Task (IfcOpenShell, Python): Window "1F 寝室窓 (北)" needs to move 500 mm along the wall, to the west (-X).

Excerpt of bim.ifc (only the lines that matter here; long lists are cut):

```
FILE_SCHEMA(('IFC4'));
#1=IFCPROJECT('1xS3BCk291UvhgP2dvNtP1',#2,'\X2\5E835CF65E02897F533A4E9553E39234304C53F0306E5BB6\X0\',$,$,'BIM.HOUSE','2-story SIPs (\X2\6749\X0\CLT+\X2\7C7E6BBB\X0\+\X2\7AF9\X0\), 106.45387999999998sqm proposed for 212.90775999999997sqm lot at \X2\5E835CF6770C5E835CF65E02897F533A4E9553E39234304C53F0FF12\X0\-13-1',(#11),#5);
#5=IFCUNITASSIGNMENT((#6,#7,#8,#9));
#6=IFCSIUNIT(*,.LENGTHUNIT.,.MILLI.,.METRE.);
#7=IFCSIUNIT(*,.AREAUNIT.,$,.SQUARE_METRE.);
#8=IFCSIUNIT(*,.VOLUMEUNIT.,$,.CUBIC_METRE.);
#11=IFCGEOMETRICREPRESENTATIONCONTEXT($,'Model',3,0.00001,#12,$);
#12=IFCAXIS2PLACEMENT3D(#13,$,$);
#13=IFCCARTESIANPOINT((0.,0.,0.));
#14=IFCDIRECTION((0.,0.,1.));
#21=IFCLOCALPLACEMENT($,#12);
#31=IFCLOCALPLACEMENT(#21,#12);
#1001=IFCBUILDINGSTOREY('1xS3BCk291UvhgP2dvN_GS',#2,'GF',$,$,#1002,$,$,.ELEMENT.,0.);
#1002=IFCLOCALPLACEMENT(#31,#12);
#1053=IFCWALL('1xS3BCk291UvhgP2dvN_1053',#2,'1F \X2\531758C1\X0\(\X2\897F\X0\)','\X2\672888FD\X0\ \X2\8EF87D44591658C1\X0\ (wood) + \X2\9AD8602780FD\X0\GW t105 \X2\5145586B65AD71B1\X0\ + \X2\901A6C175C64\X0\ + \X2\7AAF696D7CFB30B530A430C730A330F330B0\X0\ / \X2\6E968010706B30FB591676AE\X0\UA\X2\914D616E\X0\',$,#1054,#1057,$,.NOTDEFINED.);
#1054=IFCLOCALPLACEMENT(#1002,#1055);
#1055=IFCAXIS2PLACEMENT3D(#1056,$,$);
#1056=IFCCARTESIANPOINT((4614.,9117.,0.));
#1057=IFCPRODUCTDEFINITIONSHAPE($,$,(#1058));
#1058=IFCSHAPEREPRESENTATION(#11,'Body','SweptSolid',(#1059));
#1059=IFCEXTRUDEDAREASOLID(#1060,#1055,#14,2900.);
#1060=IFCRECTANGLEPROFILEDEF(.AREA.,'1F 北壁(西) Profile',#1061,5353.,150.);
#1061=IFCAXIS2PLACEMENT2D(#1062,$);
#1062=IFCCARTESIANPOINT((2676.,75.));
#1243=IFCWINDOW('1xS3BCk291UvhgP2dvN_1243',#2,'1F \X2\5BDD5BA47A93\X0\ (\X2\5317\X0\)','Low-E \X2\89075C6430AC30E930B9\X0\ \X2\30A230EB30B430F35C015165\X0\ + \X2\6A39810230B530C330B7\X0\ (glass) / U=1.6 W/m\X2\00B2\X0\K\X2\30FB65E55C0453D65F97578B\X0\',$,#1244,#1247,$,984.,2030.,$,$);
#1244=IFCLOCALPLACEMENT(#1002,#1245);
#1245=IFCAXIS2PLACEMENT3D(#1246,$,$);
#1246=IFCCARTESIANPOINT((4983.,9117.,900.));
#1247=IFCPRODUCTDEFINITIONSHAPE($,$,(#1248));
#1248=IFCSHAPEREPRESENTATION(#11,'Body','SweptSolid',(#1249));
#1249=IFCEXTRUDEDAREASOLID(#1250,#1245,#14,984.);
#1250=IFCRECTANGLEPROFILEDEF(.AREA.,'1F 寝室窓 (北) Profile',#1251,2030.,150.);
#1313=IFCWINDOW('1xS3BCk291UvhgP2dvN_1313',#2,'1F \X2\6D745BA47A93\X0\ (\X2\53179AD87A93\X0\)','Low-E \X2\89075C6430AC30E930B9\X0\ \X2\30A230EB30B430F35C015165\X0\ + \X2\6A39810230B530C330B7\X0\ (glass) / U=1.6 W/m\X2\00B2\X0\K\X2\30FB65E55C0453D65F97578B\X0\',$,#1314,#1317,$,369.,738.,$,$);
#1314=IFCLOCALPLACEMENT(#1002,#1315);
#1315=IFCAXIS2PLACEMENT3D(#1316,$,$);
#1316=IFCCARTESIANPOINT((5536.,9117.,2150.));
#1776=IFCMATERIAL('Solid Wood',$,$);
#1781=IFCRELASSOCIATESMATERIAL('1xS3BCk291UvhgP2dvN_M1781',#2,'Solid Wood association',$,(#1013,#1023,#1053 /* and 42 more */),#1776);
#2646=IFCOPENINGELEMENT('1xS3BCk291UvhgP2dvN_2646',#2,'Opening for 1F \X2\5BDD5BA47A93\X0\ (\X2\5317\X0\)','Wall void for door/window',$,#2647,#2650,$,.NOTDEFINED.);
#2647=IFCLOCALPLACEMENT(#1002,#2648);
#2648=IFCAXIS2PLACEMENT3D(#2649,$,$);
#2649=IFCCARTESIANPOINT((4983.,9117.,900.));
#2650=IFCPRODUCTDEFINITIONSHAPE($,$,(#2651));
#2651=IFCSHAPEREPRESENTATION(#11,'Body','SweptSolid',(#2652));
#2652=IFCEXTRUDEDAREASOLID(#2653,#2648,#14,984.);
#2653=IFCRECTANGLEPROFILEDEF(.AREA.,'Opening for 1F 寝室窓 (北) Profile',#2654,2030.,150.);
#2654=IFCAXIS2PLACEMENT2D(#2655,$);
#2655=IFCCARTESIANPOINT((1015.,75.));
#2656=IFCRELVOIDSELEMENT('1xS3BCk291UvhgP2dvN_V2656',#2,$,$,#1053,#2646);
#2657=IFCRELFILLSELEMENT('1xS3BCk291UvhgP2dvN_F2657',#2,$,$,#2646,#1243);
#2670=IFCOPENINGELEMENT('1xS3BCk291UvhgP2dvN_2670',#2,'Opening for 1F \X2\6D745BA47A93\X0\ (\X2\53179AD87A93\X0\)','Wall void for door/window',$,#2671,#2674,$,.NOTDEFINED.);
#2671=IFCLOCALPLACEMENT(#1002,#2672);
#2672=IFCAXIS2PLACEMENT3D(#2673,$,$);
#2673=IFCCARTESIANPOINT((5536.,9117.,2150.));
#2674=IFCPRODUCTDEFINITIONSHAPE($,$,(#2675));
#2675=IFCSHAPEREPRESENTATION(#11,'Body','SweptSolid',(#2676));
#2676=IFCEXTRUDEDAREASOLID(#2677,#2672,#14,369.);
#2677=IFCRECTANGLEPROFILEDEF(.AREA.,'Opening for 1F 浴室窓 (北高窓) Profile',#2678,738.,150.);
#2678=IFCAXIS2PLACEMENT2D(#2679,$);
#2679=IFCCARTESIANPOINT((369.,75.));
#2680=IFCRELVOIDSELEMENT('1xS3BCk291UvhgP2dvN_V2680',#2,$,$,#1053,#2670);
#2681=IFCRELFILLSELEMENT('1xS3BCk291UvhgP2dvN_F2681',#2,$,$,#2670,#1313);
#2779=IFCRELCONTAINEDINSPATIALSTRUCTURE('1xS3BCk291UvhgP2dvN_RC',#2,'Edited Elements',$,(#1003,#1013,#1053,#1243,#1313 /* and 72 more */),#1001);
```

```python
import ifcopenshell
import ifcopenshell.api.geometry
import ifcopenshell.util.placement
import ifcopenshell.util.unit

model = ifcopenshell.open("bim.ifc")
unit_scale = ifcopenshell.util.unit.calculate_unit_scale(model)

window = model.by_id(1243)
opening = window.FillsVoids[0].RelatingOpeningElement
wall = opening.VoidsElements[0].RelatingBuildingElement

wall_matrix = ifcopenshell.util.placement.get_local_placement(wall.ObjectPlacement)
shift = wall_matrix[:3, 0] * -0.5 / unit_scale
before = ifcopenshell.util.placement.get_local_placement(window.ObjectPlacement)[:3, 3].copy()

# The window is not placed relative to its opening, so move both.
for product in (opening, window):
    matrix = ifcopenshell.util.placement.get_local_placement(product.ObjectPlacement)
    matrix[:3, 3] += shift
    ifcopenshell.api.geometry.edit_object_placement(model, product=product, matrix=matrix, is_si=False)

after = ifcopenshell.util.placement.get_local_placement(window.ObjectPlacement)[:3, 3]
print("window moved by", (after - before).round(3) + 0.0)

model.write("bim_rev.ifc")
```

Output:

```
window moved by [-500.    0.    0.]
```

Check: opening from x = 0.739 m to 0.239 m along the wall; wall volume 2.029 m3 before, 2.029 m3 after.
